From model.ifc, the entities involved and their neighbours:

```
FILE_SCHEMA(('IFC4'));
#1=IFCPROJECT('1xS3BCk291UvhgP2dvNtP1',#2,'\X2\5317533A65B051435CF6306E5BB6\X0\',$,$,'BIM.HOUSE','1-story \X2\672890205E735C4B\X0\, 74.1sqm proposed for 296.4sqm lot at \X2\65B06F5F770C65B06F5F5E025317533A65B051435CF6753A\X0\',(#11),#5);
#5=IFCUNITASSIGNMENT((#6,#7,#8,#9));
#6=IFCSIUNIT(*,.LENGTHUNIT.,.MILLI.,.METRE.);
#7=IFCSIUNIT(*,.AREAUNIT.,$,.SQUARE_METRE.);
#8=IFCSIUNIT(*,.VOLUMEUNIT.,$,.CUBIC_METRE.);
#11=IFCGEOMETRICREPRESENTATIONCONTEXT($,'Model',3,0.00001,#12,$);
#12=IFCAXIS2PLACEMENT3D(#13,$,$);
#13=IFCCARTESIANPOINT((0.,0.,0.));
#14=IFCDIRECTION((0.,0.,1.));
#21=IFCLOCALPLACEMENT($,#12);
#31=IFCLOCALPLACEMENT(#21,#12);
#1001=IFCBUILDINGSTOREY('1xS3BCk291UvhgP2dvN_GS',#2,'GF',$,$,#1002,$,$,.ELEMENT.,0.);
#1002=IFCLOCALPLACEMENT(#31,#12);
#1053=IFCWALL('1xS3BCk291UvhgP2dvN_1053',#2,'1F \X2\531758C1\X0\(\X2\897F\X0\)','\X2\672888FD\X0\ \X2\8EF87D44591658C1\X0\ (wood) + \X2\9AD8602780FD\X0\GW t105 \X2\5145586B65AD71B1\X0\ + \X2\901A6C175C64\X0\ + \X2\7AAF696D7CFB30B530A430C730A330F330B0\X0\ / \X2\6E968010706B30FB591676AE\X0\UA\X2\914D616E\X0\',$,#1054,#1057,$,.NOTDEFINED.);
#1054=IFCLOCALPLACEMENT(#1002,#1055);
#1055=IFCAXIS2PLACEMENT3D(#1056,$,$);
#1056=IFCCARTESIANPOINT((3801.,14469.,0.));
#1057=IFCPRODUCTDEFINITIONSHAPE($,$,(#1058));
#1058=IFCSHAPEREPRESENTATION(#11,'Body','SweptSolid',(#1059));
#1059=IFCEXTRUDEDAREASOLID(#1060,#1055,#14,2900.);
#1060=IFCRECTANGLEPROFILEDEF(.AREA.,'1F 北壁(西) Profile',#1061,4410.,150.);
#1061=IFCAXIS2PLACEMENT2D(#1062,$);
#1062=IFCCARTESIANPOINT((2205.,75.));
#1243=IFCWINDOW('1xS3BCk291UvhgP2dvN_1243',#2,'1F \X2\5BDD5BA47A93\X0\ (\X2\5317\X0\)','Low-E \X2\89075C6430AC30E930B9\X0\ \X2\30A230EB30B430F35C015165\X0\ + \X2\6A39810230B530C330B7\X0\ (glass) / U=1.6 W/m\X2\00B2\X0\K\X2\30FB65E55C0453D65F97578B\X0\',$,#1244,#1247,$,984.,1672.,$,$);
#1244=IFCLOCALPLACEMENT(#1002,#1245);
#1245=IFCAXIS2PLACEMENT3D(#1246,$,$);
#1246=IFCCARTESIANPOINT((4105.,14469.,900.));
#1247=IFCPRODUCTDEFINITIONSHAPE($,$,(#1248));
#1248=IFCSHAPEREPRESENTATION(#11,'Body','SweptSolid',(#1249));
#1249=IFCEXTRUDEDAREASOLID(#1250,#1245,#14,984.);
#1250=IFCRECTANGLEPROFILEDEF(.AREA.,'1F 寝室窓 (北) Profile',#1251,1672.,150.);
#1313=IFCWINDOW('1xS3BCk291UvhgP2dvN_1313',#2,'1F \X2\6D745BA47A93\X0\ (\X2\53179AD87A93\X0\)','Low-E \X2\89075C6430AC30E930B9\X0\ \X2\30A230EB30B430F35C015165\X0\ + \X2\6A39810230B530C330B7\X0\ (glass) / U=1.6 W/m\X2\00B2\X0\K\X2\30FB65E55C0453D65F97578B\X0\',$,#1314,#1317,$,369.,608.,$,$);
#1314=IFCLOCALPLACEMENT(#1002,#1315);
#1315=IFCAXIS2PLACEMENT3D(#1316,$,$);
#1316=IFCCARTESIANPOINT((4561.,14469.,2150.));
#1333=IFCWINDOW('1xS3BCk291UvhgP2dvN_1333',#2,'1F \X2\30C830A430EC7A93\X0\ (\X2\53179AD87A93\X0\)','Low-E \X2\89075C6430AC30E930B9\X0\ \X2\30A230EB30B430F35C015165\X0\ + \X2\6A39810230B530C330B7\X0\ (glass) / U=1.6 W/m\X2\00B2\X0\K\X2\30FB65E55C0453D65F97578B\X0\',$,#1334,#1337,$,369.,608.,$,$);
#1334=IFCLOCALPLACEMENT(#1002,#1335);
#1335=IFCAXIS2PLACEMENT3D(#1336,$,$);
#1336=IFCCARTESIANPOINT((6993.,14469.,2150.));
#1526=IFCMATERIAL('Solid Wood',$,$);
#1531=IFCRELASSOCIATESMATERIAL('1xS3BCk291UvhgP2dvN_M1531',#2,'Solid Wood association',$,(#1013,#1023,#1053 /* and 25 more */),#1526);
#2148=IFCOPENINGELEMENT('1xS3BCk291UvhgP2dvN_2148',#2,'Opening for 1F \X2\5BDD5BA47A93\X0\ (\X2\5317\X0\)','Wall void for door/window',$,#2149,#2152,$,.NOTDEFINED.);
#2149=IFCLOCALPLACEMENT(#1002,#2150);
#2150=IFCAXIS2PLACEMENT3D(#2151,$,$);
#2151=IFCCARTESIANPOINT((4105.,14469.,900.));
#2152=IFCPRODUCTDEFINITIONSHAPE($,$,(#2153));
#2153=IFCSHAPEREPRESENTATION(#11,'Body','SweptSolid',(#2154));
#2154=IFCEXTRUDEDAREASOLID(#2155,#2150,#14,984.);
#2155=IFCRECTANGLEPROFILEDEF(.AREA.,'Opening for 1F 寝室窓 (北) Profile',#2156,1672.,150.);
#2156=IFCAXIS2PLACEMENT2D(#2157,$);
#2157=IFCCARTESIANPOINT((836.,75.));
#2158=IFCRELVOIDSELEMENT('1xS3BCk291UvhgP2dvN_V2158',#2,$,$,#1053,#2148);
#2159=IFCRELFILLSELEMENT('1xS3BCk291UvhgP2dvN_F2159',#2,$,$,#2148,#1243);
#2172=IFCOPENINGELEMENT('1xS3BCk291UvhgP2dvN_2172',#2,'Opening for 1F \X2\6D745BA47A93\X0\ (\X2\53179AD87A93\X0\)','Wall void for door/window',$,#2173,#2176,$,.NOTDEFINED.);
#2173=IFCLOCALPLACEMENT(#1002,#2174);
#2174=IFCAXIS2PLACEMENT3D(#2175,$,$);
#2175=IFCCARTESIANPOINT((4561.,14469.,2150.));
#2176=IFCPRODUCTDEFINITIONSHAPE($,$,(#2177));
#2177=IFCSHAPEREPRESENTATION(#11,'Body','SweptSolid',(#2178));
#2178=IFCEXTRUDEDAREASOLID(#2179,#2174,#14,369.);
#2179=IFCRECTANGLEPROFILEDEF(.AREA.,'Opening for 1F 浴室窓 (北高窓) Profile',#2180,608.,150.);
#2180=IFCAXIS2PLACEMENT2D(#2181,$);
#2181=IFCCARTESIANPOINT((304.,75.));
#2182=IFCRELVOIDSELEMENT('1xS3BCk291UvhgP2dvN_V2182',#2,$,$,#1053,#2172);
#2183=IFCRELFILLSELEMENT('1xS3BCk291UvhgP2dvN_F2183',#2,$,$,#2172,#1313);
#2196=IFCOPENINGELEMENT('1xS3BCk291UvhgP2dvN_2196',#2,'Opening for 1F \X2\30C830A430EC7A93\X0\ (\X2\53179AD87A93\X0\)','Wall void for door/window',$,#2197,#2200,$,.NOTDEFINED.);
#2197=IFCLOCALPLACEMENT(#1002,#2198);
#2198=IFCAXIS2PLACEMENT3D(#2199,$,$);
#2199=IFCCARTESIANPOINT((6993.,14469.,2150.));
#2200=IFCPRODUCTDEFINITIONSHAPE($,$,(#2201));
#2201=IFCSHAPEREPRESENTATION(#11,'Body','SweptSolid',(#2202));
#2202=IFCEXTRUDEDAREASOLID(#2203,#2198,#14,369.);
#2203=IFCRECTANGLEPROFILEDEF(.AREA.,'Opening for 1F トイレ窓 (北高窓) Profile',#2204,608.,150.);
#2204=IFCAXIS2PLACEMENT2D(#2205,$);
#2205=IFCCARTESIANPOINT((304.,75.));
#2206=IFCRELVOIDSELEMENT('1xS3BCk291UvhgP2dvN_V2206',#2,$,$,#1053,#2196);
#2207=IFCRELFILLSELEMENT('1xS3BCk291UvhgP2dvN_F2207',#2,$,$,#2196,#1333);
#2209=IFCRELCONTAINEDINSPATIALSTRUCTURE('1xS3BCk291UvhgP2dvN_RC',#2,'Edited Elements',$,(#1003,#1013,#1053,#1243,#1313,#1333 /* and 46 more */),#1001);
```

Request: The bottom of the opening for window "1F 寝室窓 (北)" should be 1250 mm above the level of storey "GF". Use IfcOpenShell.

```python
import numpy as np
import ifcopenshell
import ifcopenshell.api.geometry
import ifcopenshell.geom
import ifcopenshell.util.element
import ifcopenshell.util.placement
import ifcopenshell.util.shape
import ifcopenshell.util.unit

model = ifcopenshell.open("model.ifc")
unit_scale = ifcopenshell.util.unit.calculate_unit_scale(model)

window = model.by_id(1243)
opening = window.FillsVoids[0].RelatingOpeningElement
storey = ifcopenshell.util.element.get_container(window, ifc_class="IfcBuildingStorey")
level = ifcopenshell.util.placement.get_local_placement(storey.ObjectPlacement)[2, 3]

# The opening's origin need not be at the sill, so measure its lowest point.
shape = ifcopenshell.geom.create_shape(ifcopenshell.geom.settings(), opening)
bottom = ifcopenshell.util.shape.get_shape_bottom_elevation(shape, shape.geometry) / unit_scale
dz = level + 1250.0 - bottom

shift = np.array([0.0, 0.0, dz])
# The window is not placed relative to its opening, so move both.
for product in (opening, window):
    matrix = ifcopenshell.util.placement.get_local_placement(product.ObjectPlacement)
    matrix[:3, 3] += shift
    ifcopenshell.api.geometry.edit_object_placement(model, product=product, matrix=matrix, is_si=False)

print(f"moved by {dz * unit_scale:+.3f} m")

model.write("model_updated.ifc")
```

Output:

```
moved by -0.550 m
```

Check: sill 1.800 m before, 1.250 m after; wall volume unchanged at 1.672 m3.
